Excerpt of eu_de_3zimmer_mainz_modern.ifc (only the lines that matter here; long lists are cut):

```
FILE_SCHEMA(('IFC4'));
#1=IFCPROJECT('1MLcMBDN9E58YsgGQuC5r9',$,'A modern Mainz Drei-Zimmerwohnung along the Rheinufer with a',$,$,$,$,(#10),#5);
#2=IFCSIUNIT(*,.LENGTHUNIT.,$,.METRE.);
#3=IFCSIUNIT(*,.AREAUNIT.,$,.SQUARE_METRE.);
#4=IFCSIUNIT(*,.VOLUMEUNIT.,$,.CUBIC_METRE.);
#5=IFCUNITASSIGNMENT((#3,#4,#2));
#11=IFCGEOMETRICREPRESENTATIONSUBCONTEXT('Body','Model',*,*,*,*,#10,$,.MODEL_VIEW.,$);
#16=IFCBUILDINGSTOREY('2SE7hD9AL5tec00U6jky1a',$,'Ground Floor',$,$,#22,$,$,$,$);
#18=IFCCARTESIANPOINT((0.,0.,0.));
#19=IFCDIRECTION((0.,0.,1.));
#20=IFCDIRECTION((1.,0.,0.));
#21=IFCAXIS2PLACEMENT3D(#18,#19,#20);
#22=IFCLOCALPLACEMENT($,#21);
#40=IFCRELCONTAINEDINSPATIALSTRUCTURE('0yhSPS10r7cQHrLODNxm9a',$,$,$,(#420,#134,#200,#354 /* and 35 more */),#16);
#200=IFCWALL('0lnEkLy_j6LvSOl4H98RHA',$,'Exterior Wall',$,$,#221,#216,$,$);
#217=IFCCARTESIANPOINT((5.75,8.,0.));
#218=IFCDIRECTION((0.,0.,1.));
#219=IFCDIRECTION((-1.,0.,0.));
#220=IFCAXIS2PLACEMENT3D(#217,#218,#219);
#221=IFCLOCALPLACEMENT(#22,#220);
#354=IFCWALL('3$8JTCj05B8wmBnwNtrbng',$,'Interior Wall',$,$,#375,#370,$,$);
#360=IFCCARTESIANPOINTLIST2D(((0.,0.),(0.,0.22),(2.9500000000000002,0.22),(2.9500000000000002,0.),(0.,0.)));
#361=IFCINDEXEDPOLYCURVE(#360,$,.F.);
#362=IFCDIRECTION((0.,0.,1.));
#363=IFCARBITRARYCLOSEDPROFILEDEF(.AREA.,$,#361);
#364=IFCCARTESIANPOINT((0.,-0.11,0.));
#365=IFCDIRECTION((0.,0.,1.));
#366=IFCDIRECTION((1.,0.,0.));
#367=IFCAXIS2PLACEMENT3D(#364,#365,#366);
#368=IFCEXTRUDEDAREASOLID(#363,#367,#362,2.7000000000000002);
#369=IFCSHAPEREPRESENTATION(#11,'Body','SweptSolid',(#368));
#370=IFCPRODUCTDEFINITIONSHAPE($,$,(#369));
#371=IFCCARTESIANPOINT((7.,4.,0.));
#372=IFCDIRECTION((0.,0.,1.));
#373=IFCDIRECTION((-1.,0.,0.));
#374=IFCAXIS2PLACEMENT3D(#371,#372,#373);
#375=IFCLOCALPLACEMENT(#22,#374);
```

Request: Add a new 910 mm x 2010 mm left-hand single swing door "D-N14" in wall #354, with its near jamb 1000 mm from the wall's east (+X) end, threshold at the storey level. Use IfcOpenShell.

```python
import numpy as np
import ifcopenshell
import ifcopenshell.api.feature
import ifcopenshell.api.geometry
import ifcopenshell.api.root
import ifcopenshell.api.spatial
import ifcopenshell.geom
import ifcopenshell.util.element
import ifcopenshell.util.placement
import ifcopenshell.util.representation
import ifcopenshell.util.shape
import ifcopenshell.util.unit

model = ifcopenshell.open("eu_de_3zimmer_mainz_modern.ifc")
unit_scale = ifcopenshell.util.unit.calculate_unit_scale(model)
settings = ifcopenshell.geom.settings()


def volume(element):
    """Net volume in cubic metres, openings subtracted."""
    shape = ifcopenshell.geom.create_shape(settings, element)
    return ifcopenshell.util.shape.get_volume(shape.geometry)


wall = model.by_guid("3$8JTCj05B8wmBnwNtrbng")
storey = ifcopenshell.util.element.get_container(wall, ifc_class="IfcBuildingStorey")
context = ifcopenshell.util.representation.get_context(model, "Model", "Body", "MODEL_VIEW")
before = volume(wall)

width, height, from_end, sill = 0.91, 2.01, 1, 0.0  # metres

# The wall runs along its own X axis, and the end named is its -X end.
wall_shape = ifcopenshell.geom.create_shape(settings, wall)
x, y, z = ifcopenshell.util.shape.get_vertices(wall_shape.geometry).T
start = x.min() + from_end
face, thickness = float(y.min()), float(y.max() - y.min())
wall_matrix = ifcopenshell.util.placement.get_local_placement(wall.ObjectPlacement)
level = ifcopenshell.util.placement.get_local_placement(storey.ObjectPlacement)[2, 3]


def in_wall(x, y):
    """Placement at x, y metres in the wall's axes, at sill height."""
    matrix = wall_matrix.copy()
    matrix[:, 3] = wall_matrix @ np.array([x / unit_scale, y / unit_scale, 0.0, 1.0])
    matrix[2, 3] = level + sill / unit_scale
    return matrix


# Opening: a box that overshoots both wall faces by 50 mm.
opening = ifcopenshell.api.root.create_entity(model, ifc_class="IfcOpeningElement", predefined_type="OPENING")
box = ifcopenshell.api.geometry.add_wall_representation(
    model, context=context, length=width, height=height, thickness=thickness + 0.1
)
ifcopenshell.api.geometry.assign_representation(model, product=opening, representation=box)
ifcopenshell.api.geometry.edit_object_placement(model, product=opening, matrix=in_wall(start, face - 0.05), is_si=False)
ifcopenshell.api.feature.add_feature(model, feature=opening, element=wall)

door = ifcopenshell.api.root.create_entity(model, ifc_class="IfcDoor", name="D-N14", predefined_type="DOOR")
door.OverallWidth, door.OverallHeight = width / unit_scale, height / unit_scale
door.OperationType = "SINGLE_SWING_LEFT"
body = ifcopenshell.api.geometry.add_door_representation(
    model,
    context=context,
    overall_width=door.OverallWidth,
    overall_height=door.OverallHeight,
    operation_type="SINGLE_SWING_LEFT",
    lining_properties={"LiningDepth": thickness / unit_scale, "ThresholdDepth": thickness / unit_scale},
)
ifcopenshell.api.geometry.assign_representation(model, product=door, representation=body)
ifcopenshell.api.spatial.assign_container(model, products=[door], relating_structure=storey)
ifcopenshell.api.feature.add_filling(model, opening=opening, element=door)

# The lining spans the wall, so the door starts at the wall face.
ifcopenshell.api.geometry.edit_object_placement(model, product=door, matrix=in_wall(start, face), is_si=False)

after = volume(wall)

print(f"wall volume {before:.3f} -> {after:.3f} m3")

model.write("eu_de_3zimmer_mainz_modern_v2.ifc")
```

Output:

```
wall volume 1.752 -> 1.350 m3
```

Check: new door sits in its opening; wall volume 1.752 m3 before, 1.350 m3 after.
